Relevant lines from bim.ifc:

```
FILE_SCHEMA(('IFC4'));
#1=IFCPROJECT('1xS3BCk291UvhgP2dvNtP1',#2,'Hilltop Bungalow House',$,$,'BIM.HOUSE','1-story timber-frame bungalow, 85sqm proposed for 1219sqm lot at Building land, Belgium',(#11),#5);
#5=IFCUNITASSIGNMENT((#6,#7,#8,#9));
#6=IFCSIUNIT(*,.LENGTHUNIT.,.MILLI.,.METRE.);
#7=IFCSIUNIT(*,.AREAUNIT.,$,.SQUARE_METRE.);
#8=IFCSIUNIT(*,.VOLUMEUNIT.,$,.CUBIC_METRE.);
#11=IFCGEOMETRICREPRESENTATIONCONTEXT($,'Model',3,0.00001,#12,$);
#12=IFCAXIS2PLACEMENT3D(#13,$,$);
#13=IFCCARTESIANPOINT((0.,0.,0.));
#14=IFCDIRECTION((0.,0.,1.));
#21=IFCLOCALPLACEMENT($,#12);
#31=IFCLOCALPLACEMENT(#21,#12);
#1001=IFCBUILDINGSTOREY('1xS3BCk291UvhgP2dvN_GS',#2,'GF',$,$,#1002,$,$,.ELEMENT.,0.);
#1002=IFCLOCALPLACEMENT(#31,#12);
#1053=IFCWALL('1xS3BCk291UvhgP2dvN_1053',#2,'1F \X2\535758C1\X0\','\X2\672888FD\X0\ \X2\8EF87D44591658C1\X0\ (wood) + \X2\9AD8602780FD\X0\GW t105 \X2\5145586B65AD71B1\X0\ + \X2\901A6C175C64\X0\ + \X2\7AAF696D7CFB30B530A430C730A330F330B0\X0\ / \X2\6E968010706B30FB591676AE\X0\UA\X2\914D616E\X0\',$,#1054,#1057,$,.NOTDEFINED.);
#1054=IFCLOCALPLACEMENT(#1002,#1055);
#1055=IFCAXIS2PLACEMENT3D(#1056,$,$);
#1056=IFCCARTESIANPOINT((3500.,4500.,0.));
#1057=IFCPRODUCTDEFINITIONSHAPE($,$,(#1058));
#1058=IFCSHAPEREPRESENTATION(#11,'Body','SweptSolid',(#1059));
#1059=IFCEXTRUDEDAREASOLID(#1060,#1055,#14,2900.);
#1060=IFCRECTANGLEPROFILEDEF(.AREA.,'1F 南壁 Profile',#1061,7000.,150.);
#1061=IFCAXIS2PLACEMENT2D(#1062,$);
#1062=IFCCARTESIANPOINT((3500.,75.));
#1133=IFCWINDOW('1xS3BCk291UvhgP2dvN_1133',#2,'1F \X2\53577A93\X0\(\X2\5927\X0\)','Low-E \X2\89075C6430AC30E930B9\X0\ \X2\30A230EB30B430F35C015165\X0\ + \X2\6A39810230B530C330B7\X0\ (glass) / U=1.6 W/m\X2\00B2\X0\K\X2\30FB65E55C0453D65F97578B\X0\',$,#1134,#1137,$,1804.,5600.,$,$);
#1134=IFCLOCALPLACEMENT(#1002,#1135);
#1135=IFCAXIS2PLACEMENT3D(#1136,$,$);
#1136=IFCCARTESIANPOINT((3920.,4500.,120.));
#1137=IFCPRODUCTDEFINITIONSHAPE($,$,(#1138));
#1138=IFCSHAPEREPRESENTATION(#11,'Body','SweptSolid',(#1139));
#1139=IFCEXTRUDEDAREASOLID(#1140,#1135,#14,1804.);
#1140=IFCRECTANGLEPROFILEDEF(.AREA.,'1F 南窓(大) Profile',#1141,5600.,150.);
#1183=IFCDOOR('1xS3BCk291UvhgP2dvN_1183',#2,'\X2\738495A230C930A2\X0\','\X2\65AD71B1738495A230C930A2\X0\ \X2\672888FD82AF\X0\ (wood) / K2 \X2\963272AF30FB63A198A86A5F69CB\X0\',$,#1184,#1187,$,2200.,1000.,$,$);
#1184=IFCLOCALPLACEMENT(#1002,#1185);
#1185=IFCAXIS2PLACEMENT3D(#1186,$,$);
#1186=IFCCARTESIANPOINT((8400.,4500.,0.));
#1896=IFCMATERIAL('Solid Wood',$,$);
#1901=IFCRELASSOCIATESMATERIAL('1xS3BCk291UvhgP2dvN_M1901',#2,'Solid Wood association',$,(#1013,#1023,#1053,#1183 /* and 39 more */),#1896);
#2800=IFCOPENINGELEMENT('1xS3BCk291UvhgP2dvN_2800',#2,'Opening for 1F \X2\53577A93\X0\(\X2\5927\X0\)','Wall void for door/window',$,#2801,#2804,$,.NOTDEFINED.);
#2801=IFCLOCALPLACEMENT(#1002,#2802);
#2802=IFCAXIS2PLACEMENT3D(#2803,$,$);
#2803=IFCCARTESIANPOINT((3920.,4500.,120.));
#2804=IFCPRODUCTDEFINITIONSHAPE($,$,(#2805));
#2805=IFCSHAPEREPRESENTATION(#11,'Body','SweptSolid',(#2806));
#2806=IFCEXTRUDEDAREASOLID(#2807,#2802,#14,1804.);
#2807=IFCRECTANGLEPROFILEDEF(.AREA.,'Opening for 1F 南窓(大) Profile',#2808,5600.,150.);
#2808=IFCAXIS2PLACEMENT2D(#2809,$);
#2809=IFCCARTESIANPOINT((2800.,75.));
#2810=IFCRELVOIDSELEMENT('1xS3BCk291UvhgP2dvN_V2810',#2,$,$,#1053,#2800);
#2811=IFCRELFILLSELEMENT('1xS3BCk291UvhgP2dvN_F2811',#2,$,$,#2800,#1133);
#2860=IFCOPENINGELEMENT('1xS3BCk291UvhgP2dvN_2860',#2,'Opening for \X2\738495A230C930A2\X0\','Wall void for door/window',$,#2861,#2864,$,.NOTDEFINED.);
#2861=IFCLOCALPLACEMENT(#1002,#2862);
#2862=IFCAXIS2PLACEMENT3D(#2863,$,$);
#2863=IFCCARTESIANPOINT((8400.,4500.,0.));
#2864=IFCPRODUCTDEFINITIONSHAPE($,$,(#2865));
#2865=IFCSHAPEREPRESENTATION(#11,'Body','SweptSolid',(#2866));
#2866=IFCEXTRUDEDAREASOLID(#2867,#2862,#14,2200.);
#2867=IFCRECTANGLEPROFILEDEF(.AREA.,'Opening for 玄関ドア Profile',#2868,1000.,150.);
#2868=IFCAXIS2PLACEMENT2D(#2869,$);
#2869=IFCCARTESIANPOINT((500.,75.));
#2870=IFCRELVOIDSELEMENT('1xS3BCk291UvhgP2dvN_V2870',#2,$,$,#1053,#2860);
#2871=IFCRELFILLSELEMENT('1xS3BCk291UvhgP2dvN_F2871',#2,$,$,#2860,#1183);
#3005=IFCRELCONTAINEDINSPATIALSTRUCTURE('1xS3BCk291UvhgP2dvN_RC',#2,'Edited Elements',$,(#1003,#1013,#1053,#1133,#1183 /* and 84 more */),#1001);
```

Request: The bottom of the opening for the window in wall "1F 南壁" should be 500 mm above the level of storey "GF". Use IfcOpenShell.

```python
import numpy as np
import ifcopenshell
import ifcopenshell.api.geometry
import ifcopenshell.geom
import ifcopenshell.util.element
import ifcopenshell.util.placement
import ifcopenshell.util.shape
import ifcopenshell.util.unit

model = ifcopenshell.open("bim.ifc")
unit_scale = ifcopenshell.util.unit.calculate_unit_scale(model)

window = model.by_guid("1xS3BCk291UvhgP2dvN_1133")
opening = window.FillsVoids[0].RelatingOpeningElement
storey = ifcopenshell.util.element.get_container(window, ifc_class="IfcBuildingStorey")
level = ifcopenshell.util.placement.get_local_placement(storey.ObjectPlacement)[2, 3]

# The opening's origin need not be at the sill, so measure its lowest point.
shape = ifcopenshell.geom.create_shape(ifcopenshell.geom.settings(), opening)
bottom = ifcopenshell.util.shape.get_shape_bottom_elevation(shape, shape.geometry) / unit_scale
dz = level + 0.5 / unit_scale - bottom

shift = np.array([0.0, 0.0, dz])
# The window is not placed relative to its opening, so move both.
for product in (opening, window):
    matrix = ifcopenshell.util.placement.get_local_placement(product.ObjectPlacement)
    matrix[:3, 3] += shift
    ifcopenshell.api.geometry.edit_object_placement(model, product=product, matrix=matrix, is_si=False)

print(f"moved by {dz * unit_scale:+.3f} m")

model.write("bim_updated.ifc")
```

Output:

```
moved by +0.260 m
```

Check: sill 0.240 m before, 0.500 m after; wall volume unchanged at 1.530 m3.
